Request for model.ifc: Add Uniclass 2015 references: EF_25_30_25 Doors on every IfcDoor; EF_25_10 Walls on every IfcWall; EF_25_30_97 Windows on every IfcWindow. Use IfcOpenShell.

First a look at what the model holds.

```python
import ifcopenshell

model = ifcopenshell.open("model.ifc")
print(model.schema)
print("classifications:", [c.Name for c in model.by_type("IfcClassification")])
for ifc_class in ("IfcDoor", "IfcRoof", "IfcStair", "IfcWall", "IfcWindow"):
    print(ifc_class, len(model.by_type(ifc_class)))
```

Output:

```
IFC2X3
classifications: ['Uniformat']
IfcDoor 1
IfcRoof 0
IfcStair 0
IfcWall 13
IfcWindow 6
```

```python
import ifcopenshell
import ifcopenshell.api.classification

model = ifcopenshell.open("model.ifc")

# IFC2X3 requires Source and Edition and has no link from the project to the system.
system = model.create_entity("IfcClassification", Source="NBS", Edition="2015", Name="Uniclass 2015")

codes = {
    "IfcDoor": ("EF_25_30_25", "Doors"),
    "IfcWall": ("EF_25_10", "Walls"),
    "IfcWindow": ("EF_25_30_97", "Windows"),
}
for ifc_class, (code, name) in codes.items():
    products = model.by_type(ifc_class)
    ifcopenshell.api.classification.add_reference(
        model, products=products, classification=system, identification=code, name=name
    )
    print(code, len(products))

model.write("model-out.ifc")
```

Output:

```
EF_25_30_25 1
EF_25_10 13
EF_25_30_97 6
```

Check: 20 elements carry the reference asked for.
